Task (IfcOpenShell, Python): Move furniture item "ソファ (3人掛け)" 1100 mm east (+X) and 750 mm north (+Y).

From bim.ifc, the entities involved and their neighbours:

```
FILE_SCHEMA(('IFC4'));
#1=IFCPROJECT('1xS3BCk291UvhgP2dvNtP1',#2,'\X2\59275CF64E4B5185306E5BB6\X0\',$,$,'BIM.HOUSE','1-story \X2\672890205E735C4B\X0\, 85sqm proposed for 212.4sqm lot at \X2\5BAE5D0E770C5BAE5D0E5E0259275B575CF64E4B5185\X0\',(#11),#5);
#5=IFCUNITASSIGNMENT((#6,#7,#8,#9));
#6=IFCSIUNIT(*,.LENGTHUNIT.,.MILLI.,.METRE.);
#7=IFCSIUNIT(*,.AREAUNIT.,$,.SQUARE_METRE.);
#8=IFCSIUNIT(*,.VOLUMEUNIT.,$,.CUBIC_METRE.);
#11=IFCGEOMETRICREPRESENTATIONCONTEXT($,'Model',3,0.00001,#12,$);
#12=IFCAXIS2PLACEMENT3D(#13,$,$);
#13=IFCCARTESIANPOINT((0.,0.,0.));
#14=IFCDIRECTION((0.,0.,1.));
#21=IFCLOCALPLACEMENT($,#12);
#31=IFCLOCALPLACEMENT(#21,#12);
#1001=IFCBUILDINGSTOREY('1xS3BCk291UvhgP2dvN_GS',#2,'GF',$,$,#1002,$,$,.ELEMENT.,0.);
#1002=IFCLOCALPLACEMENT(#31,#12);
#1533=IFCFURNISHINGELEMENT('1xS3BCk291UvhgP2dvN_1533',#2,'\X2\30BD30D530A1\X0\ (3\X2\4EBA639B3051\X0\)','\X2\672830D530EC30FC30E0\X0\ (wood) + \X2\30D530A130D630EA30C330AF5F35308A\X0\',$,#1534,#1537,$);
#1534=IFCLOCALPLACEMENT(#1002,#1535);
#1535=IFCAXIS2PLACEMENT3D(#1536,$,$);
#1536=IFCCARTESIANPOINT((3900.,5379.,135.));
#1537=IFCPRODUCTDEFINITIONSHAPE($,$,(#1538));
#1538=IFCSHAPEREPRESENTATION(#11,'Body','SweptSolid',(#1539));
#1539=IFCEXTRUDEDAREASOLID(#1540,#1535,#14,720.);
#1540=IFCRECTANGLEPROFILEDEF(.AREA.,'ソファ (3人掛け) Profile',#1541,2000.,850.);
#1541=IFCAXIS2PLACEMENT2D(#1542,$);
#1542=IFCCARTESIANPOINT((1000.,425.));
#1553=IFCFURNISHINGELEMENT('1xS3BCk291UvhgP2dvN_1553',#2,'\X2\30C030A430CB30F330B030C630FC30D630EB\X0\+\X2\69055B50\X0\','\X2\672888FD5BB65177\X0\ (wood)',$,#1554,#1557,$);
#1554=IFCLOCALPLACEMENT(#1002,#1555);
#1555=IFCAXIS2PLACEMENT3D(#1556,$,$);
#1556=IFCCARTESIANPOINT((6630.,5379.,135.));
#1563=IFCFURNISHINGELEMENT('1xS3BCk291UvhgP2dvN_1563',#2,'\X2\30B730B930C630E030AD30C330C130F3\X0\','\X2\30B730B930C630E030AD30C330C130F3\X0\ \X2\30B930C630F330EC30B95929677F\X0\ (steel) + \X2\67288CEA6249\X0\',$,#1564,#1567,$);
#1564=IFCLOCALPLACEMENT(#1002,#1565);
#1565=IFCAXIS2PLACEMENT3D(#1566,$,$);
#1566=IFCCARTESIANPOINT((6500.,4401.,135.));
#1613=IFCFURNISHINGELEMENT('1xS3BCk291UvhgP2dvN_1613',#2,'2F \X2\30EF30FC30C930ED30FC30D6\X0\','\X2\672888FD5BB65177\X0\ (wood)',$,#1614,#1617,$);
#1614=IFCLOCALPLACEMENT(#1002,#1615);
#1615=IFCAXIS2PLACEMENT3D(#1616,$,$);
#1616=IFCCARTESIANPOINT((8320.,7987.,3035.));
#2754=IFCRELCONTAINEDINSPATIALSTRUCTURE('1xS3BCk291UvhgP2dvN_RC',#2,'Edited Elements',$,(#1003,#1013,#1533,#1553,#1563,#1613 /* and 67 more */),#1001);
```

```python
import ifcopenshell
import ifcopenshell.api.geometry
import ifcopenshell.util.placement

model = ifcopenshell.open("bim.ifc")

item = model.by_id(1533)
matrix = ifcopenshell.util.placement.get_local_placement(item.ObjectPlacement)
matrix[0, 3] += 1100.0
matrix[1, 3] += 750.0
ifcopenshell.api.geometry.edit_object_placement(model, product=item, matrix=matrix, is_si=False)

print(ifcopenshell.util.placement.get_local_placement(item.ObjectPlacement).round(3) + 0.0)

model.write("bim_edited.ifc")
```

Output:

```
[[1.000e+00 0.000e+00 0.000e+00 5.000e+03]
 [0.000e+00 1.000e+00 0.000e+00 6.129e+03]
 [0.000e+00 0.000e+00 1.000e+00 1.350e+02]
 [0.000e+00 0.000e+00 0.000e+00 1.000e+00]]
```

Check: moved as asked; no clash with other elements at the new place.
